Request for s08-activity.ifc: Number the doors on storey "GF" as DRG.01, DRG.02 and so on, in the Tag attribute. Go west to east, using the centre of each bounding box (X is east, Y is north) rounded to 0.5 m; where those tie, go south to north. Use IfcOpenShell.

First a look at what the model holds.

```python
import ifcopenshell
import ifcopenshell.util.element
import ifcopenshell.util.placement

model = ifcopenshell.open("s08-activity.ifc")
print(model.schema)
storey = next(s for s in model.by_type("IfcBuildingStorey") if s.Name == "GF")
doors = [e for e in ifcopenshell.util.element.get_decomposition(storey) if e.is_a("IfcDoor")]
for e in sorted(doors, key=lambda e: e.id()):
    origin = ifcopenshell.util.placement.get_local_placement(e.ObjectPlacement)[:3, 3]
    print(e.id(), e.Tag, e.Name, origin.round(2) + 0.0, sep=" | ")
```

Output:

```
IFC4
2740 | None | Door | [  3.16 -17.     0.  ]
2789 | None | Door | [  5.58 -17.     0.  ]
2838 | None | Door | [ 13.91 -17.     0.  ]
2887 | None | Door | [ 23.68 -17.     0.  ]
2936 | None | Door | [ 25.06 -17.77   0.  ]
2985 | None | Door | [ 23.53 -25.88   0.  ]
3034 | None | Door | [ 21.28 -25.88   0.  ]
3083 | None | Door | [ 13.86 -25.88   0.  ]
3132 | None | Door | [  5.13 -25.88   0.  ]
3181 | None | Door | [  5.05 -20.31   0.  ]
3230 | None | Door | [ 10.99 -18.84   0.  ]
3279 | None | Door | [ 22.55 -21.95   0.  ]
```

```python
import ifcopenshell
import ifcopenshell.geom
import ifcopenshell.util.element
import ifcopenshell.util.shape

model = ifcopenshell.open("s08-activity.ifc")
settings = ifcopenshell.geom.settings()
settings.set("use-world-coords", True)


def centre(element):
    shape = ifcopenshell.geom.create_shape(settings, element)
    return ifcopenshell.util.shape.get_bbox_centroid(shape.geometry)


storey = next(s for s in model.by_type("IfcBuildingStorey") if s.Name == "GF")
doors = [e for e in ifcopenshell.util.element.get_decomposition(storey) if e.is_a("IfcDoor")]

# Insertion points can sit at a corner or the storey origin, so sort by the geometry (in metres).
centres = {e: centre(e) for e in doors}
doors.sort(key=lambda e: (round(centres[e][0] / 0.5), centres[e][1]))

for i, e in enumerate(doors, start=1):
    number = f"DRG.{i:02d}"
    e.Tag = number
    print(e.id(), number)

model.write("s08-activity_v2.ifc")
```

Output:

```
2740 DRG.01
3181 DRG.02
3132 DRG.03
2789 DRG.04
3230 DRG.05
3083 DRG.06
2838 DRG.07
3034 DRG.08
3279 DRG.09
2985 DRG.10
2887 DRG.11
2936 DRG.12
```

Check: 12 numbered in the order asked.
